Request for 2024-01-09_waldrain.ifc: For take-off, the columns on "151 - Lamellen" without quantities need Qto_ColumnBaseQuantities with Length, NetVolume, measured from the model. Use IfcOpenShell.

First a look at what the model holds.

```python
import ifcopenshell
import ifcopenshell.util.element
import ifcopenshell.util.unit

model = ifcopenshell.open("2024-01-09_waldrain.ifc")
print(model.schema)
for unit_type in ("LENGTHUNIT", "AREAUNIT", "VOLUMEUNIT"):
    print(unit_type, ifcopenshell.util.unit.calculate_unit_scale(model, unit_type))
storey = next(s for s in model.by_type("IfcBuildingStorey") if s.Name == "151 - Lamellen")
columns = [e for e in ifcopenshell.util.element.get_decomposition(storey) if e.is_a("IfcColumn")]
for e in sorted(columns, key=lambda e: e.id()):
    print(e.id(), e.is_a(), e.Name, list(ifcopenshell.util.element.get_psets(e, qtos_only=True)), sep=" | ")
```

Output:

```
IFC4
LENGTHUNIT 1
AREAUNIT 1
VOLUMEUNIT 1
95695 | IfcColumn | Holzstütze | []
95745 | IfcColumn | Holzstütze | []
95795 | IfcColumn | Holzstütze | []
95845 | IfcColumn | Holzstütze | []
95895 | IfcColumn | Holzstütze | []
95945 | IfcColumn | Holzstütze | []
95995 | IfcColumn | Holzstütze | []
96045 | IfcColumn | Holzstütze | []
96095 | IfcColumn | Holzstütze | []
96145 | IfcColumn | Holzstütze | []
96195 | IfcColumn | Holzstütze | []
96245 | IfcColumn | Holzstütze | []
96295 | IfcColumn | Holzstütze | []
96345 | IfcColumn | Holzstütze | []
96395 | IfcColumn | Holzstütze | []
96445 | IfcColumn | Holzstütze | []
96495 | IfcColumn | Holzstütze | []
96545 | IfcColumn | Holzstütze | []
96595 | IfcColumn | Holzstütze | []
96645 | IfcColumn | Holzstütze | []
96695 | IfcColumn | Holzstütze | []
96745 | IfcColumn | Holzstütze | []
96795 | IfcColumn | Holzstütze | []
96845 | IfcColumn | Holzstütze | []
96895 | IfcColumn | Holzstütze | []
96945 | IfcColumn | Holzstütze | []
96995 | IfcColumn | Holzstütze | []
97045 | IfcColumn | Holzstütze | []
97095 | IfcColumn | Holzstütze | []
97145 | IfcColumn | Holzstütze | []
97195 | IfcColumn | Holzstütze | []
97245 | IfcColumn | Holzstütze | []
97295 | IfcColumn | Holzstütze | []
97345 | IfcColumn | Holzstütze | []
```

```python
import ifcopenshell
import ifcopenshell.api.pset
import ifcopenshell.geom
import ifcopenshell.util.element
import ifcopenshell.util.shape
import ifcopenshell.util.unit

model = ifcopenshell.open("2024-01-09_waldrain.ifc")
unit_scale = ifcopenshell.util.unit.calculate_unit_scale(model)
volume_scale = ifcopenshell.util.unit.calculate_unit_scale(model, "VOLUMEUNIT")
settings = ifcopenshell.geom.settings()

storey = next(s for s in model.by_type("IfcBuildingStorey") if s.Name == "151 - Lamellen")
columns = [e for e in ifcopenshell.util.element.get_decomposition(storey) if e.is_a("IfcColumn")]

for e in sorted(columns, key=lambda e: e.id()):
    if ifcopenshell.util.element.get_psets(e, qtos_only=True, should_inherit=False):
        continue
    # Geometry comes back in metres, in the element's own axes.
    shape = ifcopenshell.geom.create_shape(settings, e)
    values = {
        "Length": ifcopenshell.util.shape.get_z(shape.geometry) / unit_scale,
        "NetVolume": ifcopenshell.util.shape.get_volume(shape.geometry) / volume_scale,
    }
    qto = ifcopenshell.api.pset.add_qto(model, product=e, name="Qto_ColumnBaseQuantities")
    ifcopenshell.api.pset.edit_qto(model, qto=qto, properties=values)
    print(e.id(), {k: round(v, 3) for k, v in values.items()})

model.write("2024-01-09_waldrain_edited.ifc")
```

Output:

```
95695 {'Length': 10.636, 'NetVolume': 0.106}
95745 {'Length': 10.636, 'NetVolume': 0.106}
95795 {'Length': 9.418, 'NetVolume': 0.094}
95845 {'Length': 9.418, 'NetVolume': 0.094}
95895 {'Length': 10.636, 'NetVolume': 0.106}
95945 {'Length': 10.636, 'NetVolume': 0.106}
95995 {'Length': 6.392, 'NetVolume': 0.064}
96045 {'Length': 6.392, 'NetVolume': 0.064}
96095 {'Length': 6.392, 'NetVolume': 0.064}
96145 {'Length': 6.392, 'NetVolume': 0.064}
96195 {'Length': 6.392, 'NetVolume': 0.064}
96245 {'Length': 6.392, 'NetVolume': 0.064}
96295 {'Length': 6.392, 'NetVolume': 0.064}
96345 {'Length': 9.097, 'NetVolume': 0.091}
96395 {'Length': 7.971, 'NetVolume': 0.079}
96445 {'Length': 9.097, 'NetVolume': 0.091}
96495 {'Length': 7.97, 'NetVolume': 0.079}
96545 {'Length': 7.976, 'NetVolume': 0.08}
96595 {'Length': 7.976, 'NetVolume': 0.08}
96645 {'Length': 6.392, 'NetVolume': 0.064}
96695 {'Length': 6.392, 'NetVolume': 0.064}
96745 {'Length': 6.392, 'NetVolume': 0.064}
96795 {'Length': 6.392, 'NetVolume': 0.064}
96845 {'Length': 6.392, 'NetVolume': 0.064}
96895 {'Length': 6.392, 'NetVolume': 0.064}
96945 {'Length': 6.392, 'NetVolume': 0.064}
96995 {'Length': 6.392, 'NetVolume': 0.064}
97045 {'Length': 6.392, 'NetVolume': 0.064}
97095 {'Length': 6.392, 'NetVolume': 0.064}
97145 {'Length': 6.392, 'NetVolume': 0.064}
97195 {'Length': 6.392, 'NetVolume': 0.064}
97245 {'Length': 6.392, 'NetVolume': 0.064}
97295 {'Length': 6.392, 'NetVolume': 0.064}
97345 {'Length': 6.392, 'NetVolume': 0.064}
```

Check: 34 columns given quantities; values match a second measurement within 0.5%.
